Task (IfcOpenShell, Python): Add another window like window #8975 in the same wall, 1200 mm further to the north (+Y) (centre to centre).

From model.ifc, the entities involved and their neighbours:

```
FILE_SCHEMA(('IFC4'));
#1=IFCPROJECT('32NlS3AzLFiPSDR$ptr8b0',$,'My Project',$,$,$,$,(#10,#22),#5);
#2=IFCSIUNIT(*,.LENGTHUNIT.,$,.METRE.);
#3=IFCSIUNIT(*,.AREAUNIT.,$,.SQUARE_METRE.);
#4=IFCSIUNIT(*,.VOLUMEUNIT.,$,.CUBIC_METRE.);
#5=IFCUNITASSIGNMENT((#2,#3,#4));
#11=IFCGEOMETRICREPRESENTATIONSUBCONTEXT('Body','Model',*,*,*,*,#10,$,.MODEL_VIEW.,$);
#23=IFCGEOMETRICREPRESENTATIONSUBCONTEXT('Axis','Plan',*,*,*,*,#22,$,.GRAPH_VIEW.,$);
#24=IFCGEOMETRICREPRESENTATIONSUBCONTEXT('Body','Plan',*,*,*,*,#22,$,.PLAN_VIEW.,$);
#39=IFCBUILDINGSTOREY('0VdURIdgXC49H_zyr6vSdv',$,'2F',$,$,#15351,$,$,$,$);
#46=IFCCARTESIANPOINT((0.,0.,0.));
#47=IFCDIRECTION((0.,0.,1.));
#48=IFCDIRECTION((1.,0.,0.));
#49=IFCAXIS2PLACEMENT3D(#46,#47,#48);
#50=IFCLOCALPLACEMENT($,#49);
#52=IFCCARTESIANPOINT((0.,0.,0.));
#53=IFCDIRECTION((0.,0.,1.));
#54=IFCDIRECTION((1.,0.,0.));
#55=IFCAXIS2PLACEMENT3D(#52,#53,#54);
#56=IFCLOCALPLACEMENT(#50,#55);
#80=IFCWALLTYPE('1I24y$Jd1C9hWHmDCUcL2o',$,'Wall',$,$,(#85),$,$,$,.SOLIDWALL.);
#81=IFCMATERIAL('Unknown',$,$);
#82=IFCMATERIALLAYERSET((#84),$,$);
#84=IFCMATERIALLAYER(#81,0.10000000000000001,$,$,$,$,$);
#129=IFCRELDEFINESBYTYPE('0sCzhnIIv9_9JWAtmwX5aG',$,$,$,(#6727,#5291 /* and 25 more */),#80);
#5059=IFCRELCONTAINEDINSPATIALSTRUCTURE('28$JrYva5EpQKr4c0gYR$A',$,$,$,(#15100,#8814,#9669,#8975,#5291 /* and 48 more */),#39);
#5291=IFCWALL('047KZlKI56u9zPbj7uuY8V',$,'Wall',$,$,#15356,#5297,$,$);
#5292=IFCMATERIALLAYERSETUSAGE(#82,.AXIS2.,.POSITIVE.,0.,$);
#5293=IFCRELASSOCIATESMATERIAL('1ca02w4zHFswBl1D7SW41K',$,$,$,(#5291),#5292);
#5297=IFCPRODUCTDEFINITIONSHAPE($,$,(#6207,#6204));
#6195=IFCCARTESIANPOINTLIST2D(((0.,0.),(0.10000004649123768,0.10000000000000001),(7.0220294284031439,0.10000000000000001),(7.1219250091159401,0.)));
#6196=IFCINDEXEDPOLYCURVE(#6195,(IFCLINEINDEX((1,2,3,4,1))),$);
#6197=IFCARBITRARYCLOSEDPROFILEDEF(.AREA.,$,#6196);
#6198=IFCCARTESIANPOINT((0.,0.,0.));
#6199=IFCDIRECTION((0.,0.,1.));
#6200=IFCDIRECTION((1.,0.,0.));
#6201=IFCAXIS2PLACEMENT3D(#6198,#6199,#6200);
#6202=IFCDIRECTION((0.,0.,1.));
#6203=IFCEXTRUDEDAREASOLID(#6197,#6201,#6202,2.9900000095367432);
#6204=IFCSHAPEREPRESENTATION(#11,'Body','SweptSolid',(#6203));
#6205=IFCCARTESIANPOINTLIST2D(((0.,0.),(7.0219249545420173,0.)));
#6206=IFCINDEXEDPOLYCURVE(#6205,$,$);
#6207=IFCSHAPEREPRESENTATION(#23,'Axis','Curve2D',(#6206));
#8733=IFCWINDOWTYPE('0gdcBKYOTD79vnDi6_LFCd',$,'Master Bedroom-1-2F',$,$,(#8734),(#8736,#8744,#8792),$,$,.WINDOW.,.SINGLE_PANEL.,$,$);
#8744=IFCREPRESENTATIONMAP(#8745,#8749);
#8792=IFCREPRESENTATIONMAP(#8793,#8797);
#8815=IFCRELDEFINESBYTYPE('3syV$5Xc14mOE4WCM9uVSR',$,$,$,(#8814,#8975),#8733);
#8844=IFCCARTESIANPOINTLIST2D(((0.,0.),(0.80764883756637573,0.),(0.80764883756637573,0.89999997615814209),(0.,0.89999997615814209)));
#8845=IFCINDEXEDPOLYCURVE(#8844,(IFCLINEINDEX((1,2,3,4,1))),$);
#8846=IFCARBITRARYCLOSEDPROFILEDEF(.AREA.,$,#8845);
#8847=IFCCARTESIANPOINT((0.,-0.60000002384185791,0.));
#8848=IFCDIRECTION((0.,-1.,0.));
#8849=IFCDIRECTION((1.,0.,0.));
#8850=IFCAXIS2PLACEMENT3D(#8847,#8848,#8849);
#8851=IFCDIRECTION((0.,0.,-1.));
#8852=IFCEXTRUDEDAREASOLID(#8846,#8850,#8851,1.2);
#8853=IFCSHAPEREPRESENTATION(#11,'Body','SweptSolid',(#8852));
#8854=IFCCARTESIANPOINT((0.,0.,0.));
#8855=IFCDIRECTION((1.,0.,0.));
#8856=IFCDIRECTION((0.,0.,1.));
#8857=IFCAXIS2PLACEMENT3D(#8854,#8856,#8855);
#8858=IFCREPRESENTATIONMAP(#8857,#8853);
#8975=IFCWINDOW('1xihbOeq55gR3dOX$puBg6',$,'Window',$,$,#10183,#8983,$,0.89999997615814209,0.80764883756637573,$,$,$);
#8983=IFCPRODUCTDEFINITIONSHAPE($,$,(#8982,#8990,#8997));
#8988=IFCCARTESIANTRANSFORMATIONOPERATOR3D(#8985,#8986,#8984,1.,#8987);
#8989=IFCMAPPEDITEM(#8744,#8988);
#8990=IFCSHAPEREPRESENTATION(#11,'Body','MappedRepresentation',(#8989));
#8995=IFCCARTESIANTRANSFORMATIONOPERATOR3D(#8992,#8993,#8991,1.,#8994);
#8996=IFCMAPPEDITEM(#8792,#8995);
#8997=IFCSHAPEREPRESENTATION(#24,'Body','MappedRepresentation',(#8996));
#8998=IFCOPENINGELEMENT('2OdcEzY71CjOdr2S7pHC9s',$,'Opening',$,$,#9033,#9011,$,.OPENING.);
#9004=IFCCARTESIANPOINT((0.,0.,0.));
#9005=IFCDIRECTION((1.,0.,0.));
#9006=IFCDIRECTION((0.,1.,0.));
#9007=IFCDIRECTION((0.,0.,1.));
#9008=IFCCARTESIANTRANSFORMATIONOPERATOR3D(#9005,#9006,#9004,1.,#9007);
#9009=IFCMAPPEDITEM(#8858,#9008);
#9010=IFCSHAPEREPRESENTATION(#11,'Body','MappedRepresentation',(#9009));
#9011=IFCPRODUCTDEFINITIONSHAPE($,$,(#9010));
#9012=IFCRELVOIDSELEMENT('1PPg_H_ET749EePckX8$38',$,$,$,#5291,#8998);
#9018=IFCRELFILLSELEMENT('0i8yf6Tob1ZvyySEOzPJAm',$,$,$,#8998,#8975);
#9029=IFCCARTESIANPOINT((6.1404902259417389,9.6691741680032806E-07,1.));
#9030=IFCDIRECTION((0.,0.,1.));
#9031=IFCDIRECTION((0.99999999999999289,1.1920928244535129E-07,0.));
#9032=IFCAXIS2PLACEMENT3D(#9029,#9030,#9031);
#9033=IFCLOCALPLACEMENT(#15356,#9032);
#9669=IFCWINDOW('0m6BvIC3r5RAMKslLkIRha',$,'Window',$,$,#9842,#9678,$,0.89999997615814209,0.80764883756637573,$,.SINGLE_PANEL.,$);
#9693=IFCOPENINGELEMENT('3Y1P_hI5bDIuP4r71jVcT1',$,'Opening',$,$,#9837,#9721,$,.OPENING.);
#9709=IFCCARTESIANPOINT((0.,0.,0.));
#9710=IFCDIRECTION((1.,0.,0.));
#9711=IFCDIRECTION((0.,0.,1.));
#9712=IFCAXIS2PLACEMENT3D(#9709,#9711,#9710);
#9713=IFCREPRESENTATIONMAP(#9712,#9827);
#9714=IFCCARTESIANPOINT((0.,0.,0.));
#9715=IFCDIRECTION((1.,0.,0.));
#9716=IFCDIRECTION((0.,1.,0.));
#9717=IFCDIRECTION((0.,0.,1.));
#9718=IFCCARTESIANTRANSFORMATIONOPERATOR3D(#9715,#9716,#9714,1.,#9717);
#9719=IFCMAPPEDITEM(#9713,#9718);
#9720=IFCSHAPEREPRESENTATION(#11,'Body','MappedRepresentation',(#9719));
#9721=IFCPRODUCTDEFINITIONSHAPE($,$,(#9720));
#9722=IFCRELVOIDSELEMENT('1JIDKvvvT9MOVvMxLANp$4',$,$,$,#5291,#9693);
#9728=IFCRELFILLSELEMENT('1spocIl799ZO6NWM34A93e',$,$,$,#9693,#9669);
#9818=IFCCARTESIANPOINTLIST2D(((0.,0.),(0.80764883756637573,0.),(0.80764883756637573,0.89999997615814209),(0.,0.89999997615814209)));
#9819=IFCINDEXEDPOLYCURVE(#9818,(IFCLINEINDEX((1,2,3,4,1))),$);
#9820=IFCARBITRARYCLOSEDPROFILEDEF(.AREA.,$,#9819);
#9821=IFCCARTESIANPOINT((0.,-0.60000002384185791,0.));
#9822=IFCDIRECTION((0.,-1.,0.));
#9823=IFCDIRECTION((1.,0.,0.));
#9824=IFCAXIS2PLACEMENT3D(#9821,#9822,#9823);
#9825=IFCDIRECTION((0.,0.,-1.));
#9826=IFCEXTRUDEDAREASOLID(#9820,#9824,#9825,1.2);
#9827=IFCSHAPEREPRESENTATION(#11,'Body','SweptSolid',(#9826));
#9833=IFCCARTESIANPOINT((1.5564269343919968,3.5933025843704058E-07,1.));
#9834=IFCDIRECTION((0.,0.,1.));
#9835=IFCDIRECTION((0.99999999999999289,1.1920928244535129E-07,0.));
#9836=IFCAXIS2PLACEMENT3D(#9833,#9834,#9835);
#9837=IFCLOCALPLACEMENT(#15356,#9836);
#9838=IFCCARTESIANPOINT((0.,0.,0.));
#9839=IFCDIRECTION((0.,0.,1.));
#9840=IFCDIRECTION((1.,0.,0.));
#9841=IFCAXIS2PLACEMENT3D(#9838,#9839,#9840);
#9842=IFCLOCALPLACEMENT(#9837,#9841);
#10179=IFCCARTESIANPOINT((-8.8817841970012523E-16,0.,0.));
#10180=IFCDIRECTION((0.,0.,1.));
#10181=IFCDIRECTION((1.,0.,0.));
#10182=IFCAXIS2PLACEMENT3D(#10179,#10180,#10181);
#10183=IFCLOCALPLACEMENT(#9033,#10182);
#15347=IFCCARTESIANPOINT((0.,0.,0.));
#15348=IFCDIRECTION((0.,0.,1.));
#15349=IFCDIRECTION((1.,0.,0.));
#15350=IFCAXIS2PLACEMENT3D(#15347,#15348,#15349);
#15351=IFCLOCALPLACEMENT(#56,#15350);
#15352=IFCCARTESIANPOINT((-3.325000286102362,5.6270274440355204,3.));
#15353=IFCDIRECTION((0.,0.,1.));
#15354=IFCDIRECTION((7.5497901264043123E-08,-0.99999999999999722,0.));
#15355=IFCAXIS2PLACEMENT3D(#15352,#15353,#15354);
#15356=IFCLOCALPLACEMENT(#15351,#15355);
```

```python
import ifcopenshell
import ifcopenshell.api.feature
import ifcopenshell.api.geometry
import ifcopenshell.api.root
import ifcopenshell.geom
import ifcopenshell.util.element
import ifcopenshell.util.placement
import ifcopenshell.util.shape

model = ifcopenshell.open("model.ifc")
settings = ifcopenshell.geom.settings()


def volume(element):
    """Net volume in cubic metres, openings subtracted."""
    shape = ifcopenshell.geom.create_shape(settings, element)
    return ifcopenshell.util.shape.get_volume(shape.geometry)


window = model.by_guid("1xihbOeq55gR3dOX$puBg6")
opening = window.FillsVoids[0].RelatingOpeningElement
wall = opening.VoidsElements[0].RelatingBuildingElement
before = volume(wall)
shift = ifcopenshell.util.placement.get_local_placement(wall.ObjectPlacement)[:3, 0] * -1.2

# copy_class copies the void relationship, type, container and properties, but no geometry.
new_opening = ifcopenshell.api.root.copy_class(model, product=opening)
new_opening.Representation = ifcopenshell.util.element.copy_deep(
    model, opening.Representation, exclude=["IfcGeometricRepresentationContext", "IfcRepresentationMap"]
)
new_window = ifcopenshell.api.root.copy_class(model, product=window)
new_window.Representation = ifcopenshell.util.element.copy_deep(
    model, window.Representation, exclude=["IfcGeometricRepresentationContext", "IfcRepresentationMap"]
)
ifcopenshell.api.feature.add_filling(model, opening=new_opening, element=new_window)

for old, new in ((opening, new_opening), (window, new_window)):
    matrix = ifcopenshell.util.placement.get_local_placement(old.ObjectPlacement)
    matrix[:3, 3] += shift
    ifcopenshell.api.geometry.edit_object_placement(model, product=new, matrix=matrix, is_si=False)

after = volume(wall)

print(f"wall volume {before:.3f} -> {after:.3f} m3")

model.write("model_rev.ifc")
```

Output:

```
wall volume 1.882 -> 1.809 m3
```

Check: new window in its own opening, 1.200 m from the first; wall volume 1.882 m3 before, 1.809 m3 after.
